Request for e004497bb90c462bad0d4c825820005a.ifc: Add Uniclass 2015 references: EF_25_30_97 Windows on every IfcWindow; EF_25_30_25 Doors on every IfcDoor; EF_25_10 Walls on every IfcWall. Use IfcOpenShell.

First a look at what the model holds.

```python
import ifcopenshell

model = ifcopenshell.open("e004497bb90c462bad0d4c825820005a.ifc")
print(model.schema)
print("classifications:", [c.Name for c in model.by_type("IfcClassification")])
for ifc_class in ("IfcDoor", "IfcRoof", "IfcStair", "IfcWall", "IfcWindow"):
    print(ifc_class, len(model.by_type(ifc_class)))
```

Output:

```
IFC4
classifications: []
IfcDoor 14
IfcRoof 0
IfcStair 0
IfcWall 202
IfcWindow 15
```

```python
import ifcopenshell
import ifcopenshell.api.classification

model = ifcopenshell.open("e004497bb90c462bad0d4c825820005a.ifc")

system = ifcopenshell.api.classification.add_classification(model, classification="Uniclass 2015")

codes = {
    "IfcWindow": ("EF_25_30_97", "Windows"),
    "IfcDoor": ("EF_25_30_25", "Doors"),
    "IfcWall": ("EF_25_10", "Walls"),
}
for ifc_class, (code, name) in codes.items():
    products = model.by_type(ifc_class)
    ifcopenshell.api.classification.add_reference(
        model, products=products, classification=system, identification=code, name=name
    )
    print(code, len(products))

model.write("e004497bb90c462bad0d4c825820005a-out.ifc")
```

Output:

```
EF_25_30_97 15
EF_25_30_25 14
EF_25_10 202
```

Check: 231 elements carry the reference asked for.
